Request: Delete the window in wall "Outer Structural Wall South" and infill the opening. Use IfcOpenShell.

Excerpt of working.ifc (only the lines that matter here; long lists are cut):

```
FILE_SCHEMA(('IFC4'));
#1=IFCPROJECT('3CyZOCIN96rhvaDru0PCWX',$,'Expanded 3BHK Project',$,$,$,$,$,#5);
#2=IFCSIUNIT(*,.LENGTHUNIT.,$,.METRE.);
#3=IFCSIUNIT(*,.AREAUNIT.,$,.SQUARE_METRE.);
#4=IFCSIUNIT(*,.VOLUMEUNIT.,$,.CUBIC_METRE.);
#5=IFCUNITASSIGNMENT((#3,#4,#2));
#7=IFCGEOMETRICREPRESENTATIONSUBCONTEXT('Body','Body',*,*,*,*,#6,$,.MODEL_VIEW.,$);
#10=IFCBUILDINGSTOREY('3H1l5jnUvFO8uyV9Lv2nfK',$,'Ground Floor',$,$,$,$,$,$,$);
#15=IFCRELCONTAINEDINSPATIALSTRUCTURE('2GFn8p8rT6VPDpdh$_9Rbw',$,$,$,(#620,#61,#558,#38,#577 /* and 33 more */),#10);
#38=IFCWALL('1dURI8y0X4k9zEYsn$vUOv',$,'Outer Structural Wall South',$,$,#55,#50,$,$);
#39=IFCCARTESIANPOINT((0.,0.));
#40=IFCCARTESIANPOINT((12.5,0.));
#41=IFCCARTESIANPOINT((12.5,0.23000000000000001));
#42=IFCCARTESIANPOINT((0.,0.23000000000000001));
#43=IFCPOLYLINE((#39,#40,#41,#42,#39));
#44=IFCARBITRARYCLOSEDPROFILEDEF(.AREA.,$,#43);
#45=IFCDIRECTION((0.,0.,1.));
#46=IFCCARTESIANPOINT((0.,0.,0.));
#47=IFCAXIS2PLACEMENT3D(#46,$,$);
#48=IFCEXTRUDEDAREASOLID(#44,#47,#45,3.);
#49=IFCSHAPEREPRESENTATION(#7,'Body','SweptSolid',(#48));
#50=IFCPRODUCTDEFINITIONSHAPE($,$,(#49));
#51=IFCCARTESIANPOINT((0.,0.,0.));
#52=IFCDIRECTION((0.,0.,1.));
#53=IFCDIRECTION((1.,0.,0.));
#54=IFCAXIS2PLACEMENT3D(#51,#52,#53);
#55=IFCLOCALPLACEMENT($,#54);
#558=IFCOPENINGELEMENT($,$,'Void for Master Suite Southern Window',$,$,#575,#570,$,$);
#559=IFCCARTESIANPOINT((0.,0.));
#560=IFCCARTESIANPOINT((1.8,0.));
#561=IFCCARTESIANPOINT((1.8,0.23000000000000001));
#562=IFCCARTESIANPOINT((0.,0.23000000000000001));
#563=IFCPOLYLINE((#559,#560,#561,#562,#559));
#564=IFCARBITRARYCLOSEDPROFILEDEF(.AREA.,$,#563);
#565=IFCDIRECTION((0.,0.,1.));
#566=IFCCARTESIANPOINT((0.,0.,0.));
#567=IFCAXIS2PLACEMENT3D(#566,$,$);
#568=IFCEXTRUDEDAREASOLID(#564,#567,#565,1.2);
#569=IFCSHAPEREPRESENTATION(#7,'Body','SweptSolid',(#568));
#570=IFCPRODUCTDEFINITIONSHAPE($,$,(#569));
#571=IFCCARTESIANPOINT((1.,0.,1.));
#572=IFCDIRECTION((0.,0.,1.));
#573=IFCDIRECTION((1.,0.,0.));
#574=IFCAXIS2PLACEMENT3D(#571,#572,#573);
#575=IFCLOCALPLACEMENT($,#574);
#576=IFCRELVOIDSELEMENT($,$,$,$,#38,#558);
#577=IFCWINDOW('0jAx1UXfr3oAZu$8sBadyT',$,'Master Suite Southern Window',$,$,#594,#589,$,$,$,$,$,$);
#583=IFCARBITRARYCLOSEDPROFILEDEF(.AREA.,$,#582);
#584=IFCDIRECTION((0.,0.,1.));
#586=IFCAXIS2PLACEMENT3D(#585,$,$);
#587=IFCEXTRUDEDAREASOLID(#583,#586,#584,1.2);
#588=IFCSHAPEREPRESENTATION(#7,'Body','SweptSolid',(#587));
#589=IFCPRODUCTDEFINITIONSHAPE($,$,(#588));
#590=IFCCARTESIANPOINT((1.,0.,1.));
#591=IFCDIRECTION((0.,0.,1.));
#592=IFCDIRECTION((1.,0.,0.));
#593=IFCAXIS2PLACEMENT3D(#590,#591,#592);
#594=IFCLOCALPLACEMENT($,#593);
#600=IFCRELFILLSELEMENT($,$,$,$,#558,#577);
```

```python
import ifcopenshell
import ifcopenshell.api.feature
import ifcopenshell.api.root
import ifcopenshell.geom
import ifcopenshell.util.shape

model = ifcopenshell.open("working.ifc")
settings = ifcopenshell.geom.settings()


def volume(element):
    """Net volume in cubic metres, openings subtracted."""
    shape = ifcopenshell.geom.create_shape(settings, element)
    return ifcopenshell.util.shape.get_volume(shape.geometry)


window = model.by_id(577)
opening = window.FillsVoids[0].RelatingOpeningElement
wall = opening.VoidsElements[0].RelatingBuildingElement
before = volume(wall)

ifcopenshell.api.root.remove_product(model, product=window)
ifcopenshell.api.feature.remove_feature(model, feature=opening)

after = volume(wall)

print(f"wall volume {before:.3f} -> {after:.3f} m3")

model.write("working-out.ifc")
```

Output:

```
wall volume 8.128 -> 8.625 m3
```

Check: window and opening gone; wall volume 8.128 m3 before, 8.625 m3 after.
